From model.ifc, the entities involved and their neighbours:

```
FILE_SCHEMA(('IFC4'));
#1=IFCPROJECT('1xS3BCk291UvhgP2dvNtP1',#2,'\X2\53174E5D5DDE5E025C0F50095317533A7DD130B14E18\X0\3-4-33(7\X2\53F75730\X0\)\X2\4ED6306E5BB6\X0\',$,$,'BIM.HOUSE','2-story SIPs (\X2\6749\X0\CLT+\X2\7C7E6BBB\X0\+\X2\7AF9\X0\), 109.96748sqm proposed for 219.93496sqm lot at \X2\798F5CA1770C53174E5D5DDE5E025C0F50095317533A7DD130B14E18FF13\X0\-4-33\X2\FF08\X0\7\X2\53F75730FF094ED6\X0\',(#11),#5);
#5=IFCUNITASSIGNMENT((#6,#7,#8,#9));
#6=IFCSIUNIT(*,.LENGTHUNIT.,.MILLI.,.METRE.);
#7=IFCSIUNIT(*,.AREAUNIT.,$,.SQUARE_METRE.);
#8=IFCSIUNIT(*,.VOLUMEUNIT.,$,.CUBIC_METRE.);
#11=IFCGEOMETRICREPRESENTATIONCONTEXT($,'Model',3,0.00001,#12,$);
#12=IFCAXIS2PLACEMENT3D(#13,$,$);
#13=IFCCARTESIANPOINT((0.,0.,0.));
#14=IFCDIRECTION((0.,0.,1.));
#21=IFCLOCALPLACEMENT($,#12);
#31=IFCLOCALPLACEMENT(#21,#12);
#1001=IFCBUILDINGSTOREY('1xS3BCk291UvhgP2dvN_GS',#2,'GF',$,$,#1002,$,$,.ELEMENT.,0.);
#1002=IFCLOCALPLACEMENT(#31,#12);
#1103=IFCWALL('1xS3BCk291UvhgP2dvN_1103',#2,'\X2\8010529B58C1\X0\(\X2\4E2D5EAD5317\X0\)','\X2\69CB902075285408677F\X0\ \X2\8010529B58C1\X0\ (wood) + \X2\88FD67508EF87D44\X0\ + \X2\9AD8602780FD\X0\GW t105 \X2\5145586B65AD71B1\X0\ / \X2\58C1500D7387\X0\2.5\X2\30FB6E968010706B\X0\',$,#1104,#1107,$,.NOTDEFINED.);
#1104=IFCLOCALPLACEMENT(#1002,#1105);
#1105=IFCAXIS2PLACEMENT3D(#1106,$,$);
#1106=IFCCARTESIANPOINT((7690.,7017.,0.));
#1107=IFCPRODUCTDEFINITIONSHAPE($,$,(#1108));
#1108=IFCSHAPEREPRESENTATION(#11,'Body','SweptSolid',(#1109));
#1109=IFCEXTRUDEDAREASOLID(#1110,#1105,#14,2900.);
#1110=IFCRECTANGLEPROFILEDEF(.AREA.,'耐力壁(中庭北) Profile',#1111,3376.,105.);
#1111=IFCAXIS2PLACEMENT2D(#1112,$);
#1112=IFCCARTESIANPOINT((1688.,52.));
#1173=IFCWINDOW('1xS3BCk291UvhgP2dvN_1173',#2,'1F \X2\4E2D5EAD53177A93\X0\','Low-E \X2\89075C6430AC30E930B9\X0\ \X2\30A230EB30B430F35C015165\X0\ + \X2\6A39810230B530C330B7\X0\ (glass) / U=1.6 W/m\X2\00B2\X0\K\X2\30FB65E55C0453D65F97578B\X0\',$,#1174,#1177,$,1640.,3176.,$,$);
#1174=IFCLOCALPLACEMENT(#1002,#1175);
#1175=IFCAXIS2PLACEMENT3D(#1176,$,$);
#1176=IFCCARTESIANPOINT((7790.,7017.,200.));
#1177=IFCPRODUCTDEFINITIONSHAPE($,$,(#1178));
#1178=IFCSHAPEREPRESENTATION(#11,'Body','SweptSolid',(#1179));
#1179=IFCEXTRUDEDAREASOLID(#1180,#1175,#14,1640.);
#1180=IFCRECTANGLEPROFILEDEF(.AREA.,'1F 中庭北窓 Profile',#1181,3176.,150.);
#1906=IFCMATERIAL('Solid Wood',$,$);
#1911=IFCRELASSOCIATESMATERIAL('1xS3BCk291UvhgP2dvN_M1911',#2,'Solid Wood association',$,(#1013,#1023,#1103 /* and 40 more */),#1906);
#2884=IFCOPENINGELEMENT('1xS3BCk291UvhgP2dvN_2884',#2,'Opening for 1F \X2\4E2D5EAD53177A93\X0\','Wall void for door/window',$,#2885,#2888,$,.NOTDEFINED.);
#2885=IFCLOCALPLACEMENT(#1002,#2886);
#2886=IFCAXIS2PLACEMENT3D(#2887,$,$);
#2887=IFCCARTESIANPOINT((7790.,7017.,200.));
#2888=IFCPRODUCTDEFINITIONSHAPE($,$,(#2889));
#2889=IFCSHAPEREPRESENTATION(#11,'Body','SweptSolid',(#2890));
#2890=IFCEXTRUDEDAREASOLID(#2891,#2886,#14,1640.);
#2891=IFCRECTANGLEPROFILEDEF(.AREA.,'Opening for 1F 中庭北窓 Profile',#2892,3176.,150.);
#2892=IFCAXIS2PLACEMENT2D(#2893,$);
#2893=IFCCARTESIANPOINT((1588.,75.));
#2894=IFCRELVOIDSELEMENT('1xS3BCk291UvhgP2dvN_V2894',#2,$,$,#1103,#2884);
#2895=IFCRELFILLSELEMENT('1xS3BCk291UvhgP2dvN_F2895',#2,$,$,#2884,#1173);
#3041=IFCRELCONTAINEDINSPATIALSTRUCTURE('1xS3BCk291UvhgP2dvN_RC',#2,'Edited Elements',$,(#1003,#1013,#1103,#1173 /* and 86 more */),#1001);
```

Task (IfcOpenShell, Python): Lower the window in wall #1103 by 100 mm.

```python
import numpy as np
import ifcopenshell
import ifcopenshell.api.geometry
import ifcopenshell.util.placement
import ifcopenshell.util.unit

model = ifcopenshell.open("model.ifc")
unit_scale = ifcopenshell.util.unit.calculate_unit_scale(model)

window = model.by_id(1173)
opening = window.FillsVoids[0].RelatingOpeningElement
dz = -100.0

shift = np.array([0.0, 0.0, dz])
# The window is not placed relative to its opening, so move both.
for product in (opening, window):
    matrix = ifcopenshell.util.placement.get_local_placement(product.ObjectPlacement)
    matrix[:3, 3] += shift
    ifcopenshell.api.geometry.edit_object_placement(model, product=product, matrix=matrix, is_si=False)

print(f"moved by {dz * unit_scale:+.3f} m")

model.write("model-out.ifc")
```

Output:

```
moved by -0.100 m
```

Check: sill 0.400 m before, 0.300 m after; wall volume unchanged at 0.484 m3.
